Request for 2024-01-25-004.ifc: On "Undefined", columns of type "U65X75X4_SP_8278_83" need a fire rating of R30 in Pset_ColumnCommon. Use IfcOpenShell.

First a look at what the model holds.

```python
import ifcopenshell
import ifcopenshell.util.element

model = ifcopenshell.open("2024-01-25-004.ifc")
print(model.schema)
storey = next(s for s in model.by_type("IfcBuildingStorey") if s.Name == "Undefined")
columns = [e for e in ifcopenshell.util.element.get_decomposition(storey) if e.is_a("IfcColumn")]
seen = {}
for e in columns:
    element_type = ifcopenshell.util.element.get_type(e)
    key = (element_type.Name if element_type != e and element_type else None, ifcopenshell.util.element.get_pset(e, "Pset_ColumnCommon", "FireRating"))
    seen[key] = seen.get(key, 0) + 1
for (name, value), count in sorted(seen.items(), key=str):
    print(count, "x", name, "|", value)
```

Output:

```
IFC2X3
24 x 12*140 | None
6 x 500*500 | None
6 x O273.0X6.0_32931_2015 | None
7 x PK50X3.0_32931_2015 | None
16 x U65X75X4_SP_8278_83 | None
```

```python
import ifcopenshell
import ifcopenshell.api.pset
import ifcopenshell.util.element

model = ifcopenshell.open("2024-01-25-004.ifc")

storey = next(s for s in model.by_type("IfcBuildingStorey") if s.Name == "Undefined")
columns = [e for e in ifcopenshell.util.element.get_decomposition(storey) if e.is_a("IfcColumn")]

count = 0
for e in columns:
    element_type = ifcopenshell.util.element.get_type(e)
    if element_type in (None, e) or element_type.Name != "U65X75X4_SP_8278_83":
        continue
    found = ifcopenshell.util.element.get_pset(e, "Pset_ColumnCommon", should_inherit=False)
    if found:
        pset = model.by_id(found["id"])
        if len(ifcopenshell.util.element.get_elements_by_pset(pset)) > 1:
            pset = ifcopenshell.api.pset.unshare_pset(model, products=[e], pset=pset)[0]
    else:
        pset = ifcopenshell.api.pset.add_pset(model, product=e, name="Pset_ColumnCommon")
    ifcopenshell.api.pset.edit_pset(model, pset=pset, properties={"FireRating": "R30"})
    count += 1

print(count, "columns updated")

model.write("2024-01-25-004_v2.ifc")
```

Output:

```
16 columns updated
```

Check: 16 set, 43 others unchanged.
